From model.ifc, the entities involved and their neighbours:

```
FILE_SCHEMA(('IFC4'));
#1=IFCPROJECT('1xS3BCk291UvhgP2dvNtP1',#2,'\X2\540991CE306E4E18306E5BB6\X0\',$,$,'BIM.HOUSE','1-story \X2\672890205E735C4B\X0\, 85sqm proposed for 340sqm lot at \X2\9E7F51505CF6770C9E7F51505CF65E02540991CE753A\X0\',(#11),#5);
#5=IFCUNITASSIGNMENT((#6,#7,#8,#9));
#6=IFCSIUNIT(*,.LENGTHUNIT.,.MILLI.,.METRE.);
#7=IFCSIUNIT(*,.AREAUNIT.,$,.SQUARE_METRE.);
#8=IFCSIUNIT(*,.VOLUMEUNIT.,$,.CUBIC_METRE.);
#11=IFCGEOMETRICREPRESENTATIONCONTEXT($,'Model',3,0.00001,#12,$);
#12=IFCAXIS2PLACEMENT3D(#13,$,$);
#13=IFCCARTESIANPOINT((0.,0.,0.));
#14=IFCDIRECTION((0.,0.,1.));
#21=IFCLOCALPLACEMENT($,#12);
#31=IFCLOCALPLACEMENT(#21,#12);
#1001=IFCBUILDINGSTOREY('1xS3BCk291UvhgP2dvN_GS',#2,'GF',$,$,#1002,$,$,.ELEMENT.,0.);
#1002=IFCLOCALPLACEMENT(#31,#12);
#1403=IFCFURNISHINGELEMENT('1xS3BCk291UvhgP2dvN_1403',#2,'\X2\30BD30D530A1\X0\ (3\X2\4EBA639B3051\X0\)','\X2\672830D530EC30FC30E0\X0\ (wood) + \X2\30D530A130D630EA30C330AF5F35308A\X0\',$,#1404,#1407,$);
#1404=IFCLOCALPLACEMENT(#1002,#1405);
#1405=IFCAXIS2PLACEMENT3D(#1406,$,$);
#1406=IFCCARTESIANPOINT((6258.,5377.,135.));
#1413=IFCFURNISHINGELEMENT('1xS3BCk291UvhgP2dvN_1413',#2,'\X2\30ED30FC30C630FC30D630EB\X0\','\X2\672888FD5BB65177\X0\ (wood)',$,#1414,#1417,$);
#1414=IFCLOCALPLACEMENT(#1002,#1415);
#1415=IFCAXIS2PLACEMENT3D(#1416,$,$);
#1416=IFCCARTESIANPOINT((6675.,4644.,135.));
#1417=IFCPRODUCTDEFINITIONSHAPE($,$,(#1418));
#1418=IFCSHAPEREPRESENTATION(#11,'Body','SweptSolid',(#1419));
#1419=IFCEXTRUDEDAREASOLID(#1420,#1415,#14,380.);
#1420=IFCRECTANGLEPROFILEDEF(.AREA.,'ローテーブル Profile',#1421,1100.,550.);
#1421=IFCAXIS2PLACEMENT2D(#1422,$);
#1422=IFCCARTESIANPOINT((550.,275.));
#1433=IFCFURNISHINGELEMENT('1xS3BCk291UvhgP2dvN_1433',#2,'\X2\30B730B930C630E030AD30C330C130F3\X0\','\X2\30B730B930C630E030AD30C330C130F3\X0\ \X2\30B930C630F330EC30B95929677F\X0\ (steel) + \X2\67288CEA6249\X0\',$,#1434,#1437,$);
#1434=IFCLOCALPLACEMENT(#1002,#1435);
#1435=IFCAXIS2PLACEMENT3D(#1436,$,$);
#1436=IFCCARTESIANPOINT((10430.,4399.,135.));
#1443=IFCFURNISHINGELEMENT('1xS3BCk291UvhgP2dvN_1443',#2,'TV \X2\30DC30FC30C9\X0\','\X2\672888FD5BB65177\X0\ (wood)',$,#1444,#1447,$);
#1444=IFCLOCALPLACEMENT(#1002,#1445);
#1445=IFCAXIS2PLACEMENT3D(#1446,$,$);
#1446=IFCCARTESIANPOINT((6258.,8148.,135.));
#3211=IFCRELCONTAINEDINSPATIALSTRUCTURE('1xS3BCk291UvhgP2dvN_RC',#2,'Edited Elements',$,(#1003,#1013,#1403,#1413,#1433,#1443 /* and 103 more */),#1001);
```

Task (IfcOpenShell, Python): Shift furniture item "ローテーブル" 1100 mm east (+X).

```python
import ifcopenshell
import ifcopenshell.api.geometry
import ifcopenshell.util.placement
import ifcopenshell.util.unit

model = ifcopenshell.open("model.ifc")
unit_scale = ifcopenshell.util.unit.calculate_unit_scale(model)

item = model.by_guid("1xS3BCk291UvhgP2dvN_1413")
matrix = ifcopenshell.util.placement.get_local_placement(item.ObjectPlacement)
matrix[0, 3] += 1.1 / unit_scale
ifcopenshell.api.geometry.edit_object_placement(model, product=item, matrix=matrix, is_si=False)

print(ifcopenshell.util.placement.get_local_placement(item.ObjectPlacement).round(3) + 0.0)

model.write("model_edited.ifc")
```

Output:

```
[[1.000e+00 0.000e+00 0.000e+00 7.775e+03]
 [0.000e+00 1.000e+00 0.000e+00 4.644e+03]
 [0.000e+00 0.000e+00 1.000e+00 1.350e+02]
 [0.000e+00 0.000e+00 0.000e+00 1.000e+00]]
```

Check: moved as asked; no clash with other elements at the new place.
